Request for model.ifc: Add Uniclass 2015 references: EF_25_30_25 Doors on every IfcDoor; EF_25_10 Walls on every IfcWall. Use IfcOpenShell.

First a look at what the model holds.

```python
import ifcopenshell

model = ifcopenshell.open("model.ifc")
print(model.schema)
print("classifications:", [c.Name for c in model.by_type("IfcClassification")])
for ifc_class in ("IfcDoor", "IfcRoof", "IfcStair", "IfcWall", "IfcWindow"):
    print(ifc_class, len(model.by_type(ifc_class)))
```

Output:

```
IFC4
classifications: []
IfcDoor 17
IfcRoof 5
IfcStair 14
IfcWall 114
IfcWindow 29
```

```python
import ifcopenshell
import ifcopenshell.api.classification

model = ifcopenshell.open("model.ifc")

system = ifcopenshell.api.classification.add_classification(model, classification="Uniclass 2015")

codes = {
    "IfcDoor": ("EF_25_30_25", "Doors"),
    "IfcWall": ("EF_25_10", "Walls"),
}
for ifc_class, (code, name) in codes.items():
    products = model.by_type(ifc_class)
    ifcopenshell.api.classification.add_reference(
        model, products=products, classification=system, identification=code, name=name
    )
    print(code, len(products))

model.write("model_updated.ifc")
```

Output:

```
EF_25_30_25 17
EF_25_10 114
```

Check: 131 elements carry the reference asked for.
